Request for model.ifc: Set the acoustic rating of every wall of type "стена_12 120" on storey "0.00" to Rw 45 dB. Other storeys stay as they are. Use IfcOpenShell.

First a look at what the model holds.

```python
import ifcopenshell
import ifcopenshell.util.element

model = ifcopenshell.open("model.ifc")
print(model.schema)
storey = next(s for s in model.by_type("IfcBuildingStorey") if s.Name == "0.00")
walls = [e for e in ifcopenshell.util.element.get_decomposition(storey) if e.is_a("IfcWall")]
seen = {}
for e in walls:
    element_type = ifcopenshell.util.element.get_type(e)
    key = (element_type.Name if element_type != e and element_type else None, ifcopenshell.util.element.get_pset(e, "Pset_WallCommon", "AcousticRating"))
    seen[key] = seen.get(key, 0) + 1
for (name, value), count in sorted(seen.items(), key=str):
    print(count, "x", name, "|", value)
```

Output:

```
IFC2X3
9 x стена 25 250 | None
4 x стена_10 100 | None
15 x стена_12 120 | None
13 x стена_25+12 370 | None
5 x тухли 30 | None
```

```python
import ifcopenshell
import ifcopenshell.api.pset
import ifcopenshell.util.element

model = ifcopenshell.open("model.ifc")

storey = next(s for s in model.by_type("IfcBuildingStorey") if s.Name == "0.00")
walls = [e for e in ifcopenshell.util.element.get_decomposition(storey) if e.is_a("IfcWall")]

count = 0
for e in walls:
    element_type = ifcopenshell.util.element.get_type(e)
    if element_type in (None, e) or element_type.Name != "стена_12 120":
        continue
    # add_pset returns the element's existing set when there is one.
    pset = ifcopenshell.api.pset.add_pset(model, product=e, name="Pset_WallCommon")
    ifcopenshell.api.pset.edit_pset(model, pset=pset, properties={"AcousticRating": "Rw 45 dB"})
    count += 1

print(count, "walls updated")

model.write("model_edited.ifc")
```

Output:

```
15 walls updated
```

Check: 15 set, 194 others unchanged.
